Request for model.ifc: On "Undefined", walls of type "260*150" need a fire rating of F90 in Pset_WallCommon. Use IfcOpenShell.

First a look at what the model holds.

```python
import ifcopenshell
import ifcopenshell.util.element

model = ifcopenshell.open("model.ifc")
print(model.schema)
storey = next(s for s in model.by_type("IfcBuildingStorey") if s.Name == "Undefined")
walls = [e for e in ifcopenshell.util.element.get_decomposition(storey) if e.is_a("IfcWall")]
seen = {}
for e in walls:
    element_type = ifcopenshell.util.element.get_type(e)
    key = (element_type.Name if element_type != e and element_type else None, ifcopenshell.util.element.get_pset(e, "Pset_WallCommon", "FireRating"))
    seen[key] = seen.get(key, 0) + 1
for (name, value), count in sorted(seen.items(), key=str):
    print(count, "x", name, "|", value)
```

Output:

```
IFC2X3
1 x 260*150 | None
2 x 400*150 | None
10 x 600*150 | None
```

```python
import ifcopenshell
import ifcopenshell.api.pset
import ifcopenshell.util.element

model = ifcopenshell.open("model.ifc")

storey = next(s for s in model.by_type("IfcBuildingStorey") if s.Name == "Undefined")
walls = [e for e in ifcopenshell.util.element.get_decomposition(storey) if e.is_a("IfcWall")]

count = 0
for e in walls:
    element_type = ifcopenshell.util.element.get_type(e)
    if element_type in (None, e) or element_type.Name != "260*150":
        continue
    found = ifcopenshell.util.element.get_pset(e, "Pset_WallCommon", should_inherit=False)
    if found:
        pset = model.by_id(found["id"])
        if len(ifcopenshell.util.element.get_elements_by_pset(pset)) > 1:
            pset = ifcopenshell.api.pset.unshare_pset(model, products=[e], pset=pset)[0]
    else:
        pset = ifcopenshell.api.pset.add_pset(model, product=e, name="Pset_WallCommon")
    ifcopenshell.api.pset.edit_pset(model, pset=pset, properties={"FireRating": "F90"})
    count += 1

print(count, "walls updated")

model.write("model_edited.ifc")
```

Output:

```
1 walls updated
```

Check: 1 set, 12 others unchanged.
